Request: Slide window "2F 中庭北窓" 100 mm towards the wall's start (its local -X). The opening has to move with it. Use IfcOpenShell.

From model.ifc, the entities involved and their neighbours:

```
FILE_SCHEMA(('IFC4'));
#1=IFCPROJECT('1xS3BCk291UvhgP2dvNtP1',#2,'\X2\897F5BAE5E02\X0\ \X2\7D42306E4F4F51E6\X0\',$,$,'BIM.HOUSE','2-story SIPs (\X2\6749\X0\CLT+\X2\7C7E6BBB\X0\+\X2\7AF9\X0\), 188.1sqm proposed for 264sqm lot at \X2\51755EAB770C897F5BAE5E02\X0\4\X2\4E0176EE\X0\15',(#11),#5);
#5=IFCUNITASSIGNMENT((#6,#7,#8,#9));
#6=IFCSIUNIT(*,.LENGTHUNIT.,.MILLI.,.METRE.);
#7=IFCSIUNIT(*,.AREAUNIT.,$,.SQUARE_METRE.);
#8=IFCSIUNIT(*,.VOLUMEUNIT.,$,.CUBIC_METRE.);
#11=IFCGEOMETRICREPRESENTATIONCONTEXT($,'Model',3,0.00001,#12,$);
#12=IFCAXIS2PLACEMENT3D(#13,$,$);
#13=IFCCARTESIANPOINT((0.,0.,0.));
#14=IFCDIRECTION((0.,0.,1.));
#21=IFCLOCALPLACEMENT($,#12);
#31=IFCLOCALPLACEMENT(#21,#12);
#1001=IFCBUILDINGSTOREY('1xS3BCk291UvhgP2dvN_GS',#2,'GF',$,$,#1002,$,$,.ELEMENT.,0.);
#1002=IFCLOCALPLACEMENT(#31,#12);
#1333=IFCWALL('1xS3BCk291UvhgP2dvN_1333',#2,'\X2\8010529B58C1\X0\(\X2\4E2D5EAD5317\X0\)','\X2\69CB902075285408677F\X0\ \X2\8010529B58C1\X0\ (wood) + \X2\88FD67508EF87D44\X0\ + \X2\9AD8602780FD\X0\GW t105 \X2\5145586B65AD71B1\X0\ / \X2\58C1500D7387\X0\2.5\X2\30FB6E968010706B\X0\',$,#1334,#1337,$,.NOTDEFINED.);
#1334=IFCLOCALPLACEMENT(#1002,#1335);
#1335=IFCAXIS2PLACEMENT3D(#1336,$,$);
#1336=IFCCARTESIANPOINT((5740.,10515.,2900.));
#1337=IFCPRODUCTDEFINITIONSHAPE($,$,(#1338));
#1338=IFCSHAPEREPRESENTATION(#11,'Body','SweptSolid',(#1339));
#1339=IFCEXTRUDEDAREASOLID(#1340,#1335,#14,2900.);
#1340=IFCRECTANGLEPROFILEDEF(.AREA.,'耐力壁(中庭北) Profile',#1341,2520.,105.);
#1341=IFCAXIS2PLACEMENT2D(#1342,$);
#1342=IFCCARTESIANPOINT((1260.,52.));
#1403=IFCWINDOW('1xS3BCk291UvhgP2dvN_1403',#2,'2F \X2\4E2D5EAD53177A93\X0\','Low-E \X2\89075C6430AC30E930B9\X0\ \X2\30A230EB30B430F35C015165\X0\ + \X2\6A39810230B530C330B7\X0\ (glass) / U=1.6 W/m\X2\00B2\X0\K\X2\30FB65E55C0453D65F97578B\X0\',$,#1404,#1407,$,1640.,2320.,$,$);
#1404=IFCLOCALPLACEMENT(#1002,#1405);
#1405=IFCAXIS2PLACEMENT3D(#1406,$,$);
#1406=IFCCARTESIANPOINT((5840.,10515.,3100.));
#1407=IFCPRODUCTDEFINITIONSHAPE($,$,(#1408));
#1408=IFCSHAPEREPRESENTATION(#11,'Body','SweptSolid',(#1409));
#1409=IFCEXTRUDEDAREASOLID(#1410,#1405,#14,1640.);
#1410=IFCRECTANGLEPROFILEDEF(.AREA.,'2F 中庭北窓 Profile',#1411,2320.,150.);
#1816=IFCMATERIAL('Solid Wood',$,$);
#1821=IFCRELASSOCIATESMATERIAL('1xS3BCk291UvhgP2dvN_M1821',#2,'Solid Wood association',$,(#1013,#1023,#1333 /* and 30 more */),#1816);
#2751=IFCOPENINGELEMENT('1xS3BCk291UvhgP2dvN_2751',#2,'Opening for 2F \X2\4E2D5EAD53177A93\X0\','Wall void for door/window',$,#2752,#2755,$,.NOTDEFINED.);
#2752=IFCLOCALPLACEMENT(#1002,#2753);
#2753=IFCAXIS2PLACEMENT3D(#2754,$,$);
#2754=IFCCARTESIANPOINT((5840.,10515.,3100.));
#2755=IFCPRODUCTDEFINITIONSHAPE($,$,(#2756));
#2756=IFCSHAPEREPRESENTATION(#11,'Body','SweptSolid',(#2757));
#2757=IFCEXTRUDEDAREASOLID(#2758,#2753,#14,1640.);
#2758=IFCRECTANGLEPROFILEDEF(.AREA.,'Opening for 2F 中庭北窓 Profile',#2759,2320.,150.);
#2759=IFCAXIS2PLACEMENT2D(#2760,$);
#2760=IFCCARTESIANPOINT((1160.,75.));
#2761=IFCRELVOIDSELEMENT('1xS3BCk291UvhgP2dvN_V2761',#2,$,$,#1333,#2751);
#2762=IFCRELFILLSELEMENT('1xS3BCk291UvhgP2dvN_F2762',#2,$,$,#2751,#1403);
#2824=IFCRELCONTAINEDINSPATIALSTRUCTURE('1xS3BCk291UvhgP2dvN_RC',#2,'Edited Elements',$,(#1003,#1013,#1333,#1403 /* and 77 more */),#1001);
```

```python
import ifcopenshell
import ifcopenshell.api.geometry
import ifcopenshell.util.placement
import ifcopenshell.util.unit

model = ifcopenshell.open("model.ifc")
unit_scale = ifcopenshell.util.unit.calculate_unit_scale(model)

window = model.by_guid("1xS3BCk291UvhgP2dvN_1403")
opening = window.FillsVoids[0].RelatingOpeningElement
wall = opening.VoidsElements[0].RelatingBuildingElement

wall_matrix = ifcopenshell.util.placement.get_local_placement(wall.ObjectPlacement)
shift = wall_matrix[:3, 0] * -0.1 / unit_scale
before = ifcopenshell.util.placement.get_local_placement(window.ObjectPlacement)[:3, 3].copy()

# The window is not placed relative to its opening, so move both.
for product in (opening, window):
    matrix = ifcopenshell.util.placement.get_local_placement(product.ObjectPlacement)
    matrix[:3, 3] += shift
    ifcopenshell.api.geometry.edit_object_placement(model, product=product, matrix=matrix, is_si=False)

after = ifcopenshell.util.placement.get_local_placement(window.ObjectPlacement)[:3, 3]
print("window moved by", (after - before).round(3) + 0.0)

model.write("model_edited.ifc")
```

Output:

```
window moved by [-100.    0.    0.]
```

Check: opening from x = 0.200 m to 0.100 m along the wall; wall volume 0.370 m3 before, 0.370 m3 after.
